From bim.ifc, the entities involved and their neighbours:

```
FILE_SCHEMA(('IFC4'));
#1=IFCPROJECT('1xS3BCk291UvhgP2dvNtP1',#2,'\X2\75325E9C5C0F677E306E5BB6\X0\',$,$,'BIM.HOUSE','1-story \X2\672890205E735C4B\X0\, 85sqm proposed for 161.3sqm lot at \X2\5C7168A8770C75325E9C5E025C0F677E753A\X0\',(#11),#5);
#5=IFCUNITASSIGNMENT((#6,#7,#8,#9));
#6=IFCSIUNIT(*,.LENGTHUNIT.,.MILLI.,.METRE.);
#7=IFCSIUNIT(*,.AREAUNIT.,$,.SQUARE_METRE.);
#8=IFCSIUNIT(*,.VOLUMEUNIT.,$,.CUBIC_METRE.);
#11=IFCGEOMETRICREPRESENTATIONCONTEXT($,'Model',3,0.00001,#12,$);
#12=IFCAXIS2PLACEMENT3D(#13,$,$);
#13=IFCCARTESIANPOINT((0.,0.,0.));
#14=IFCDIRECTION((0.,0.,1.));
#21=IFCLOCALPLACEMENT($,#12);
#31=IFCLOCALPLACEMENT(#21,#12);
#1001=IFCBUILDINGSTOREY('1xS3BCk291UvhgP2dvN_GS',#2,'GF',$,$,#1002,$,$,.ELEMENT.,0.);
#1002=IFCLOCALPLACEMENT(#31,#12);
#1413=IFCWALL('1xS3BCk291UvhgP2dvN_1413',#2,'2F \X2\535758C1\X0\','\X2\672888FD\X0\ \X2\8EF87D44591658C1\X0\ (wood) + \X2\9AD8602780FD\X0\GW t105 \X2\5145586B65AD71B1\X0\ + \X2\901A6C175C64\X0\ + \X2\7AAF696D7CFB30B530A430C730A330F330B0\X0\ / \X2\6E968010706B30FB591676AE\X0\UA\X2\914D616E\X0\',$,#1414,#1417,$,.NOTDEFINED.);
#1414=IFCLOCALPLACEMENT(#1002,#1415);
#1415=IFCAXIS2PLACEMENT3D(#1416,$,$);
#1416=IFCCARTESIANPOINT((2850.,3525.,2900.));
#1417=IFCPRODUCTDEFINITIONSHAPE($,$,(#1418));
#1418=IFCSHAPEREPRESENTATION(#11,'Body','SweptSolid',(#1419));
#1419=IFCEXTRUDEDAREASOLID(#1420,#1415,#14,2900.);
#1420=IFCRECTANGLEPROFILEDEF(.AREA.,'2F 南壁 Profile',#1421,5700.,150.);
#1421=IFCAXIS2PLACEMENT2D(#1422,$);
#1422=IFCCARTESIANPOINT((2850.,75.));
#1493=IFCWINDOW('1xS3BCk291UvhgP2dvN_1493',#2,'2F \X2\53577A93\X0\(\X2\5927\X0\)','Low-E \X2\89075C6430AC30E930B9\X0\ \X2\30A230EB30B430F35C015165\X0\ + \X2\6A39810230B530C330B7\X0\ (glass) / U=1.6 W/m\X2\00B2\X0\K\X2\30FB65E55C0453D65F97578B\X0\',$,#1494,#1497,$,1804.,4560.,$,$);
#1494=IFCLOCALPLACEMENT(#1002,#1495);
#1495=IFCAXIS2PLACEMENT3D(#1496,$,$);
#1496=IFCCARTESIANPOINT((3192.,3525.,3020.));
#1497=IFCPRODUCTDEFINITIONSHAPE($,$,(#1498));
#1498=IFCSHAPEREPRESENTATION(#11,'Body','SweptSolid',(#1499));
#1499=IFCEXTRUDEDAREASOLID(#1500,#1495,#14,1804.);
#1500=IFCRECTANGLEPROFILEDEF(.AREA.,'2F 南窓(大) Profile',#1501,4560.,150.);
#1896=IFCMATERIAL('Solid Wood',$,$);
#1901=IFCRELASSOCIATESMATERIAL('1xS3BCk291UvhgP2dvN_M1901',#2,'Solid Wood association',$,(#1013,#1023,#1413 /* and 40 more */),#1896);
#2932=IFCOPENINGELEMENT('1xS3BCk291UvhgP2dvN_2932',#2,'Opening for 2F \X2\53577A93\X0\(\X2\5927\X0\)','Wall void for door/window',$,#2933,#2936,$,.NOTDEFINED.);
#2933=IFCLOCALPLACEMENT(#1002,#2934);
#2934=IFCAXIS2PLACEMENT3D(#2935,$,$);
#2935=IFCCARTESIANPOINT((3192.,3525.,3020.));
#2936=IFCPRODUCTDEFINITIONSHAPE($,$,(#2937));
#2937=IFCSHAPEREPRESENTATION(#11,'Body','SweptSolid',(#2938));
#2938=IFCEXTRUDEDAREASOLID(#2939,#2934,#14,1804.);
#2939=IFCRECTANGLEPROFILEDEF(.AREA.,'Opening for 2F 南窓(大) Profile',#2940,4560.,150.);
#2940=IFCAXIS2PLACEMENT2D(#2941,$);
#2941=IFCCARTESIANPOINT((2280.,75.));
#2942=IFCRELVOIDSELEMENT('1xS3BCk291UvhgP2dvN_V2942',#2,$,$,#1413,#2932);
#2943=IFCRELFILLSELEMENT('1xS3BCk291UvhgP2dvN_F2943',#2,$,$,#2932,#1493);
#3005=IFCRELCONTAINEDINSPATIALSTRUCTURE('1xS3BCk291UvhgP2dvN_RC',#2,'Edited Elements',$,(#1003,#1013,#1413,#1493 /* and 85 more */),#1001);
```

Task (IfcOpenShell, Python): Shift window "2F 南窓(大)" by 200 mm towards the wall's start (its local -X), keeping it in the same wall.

```python
import ifcopenshell
import ifcopenshell.api.geometry
import ifcopenshell.util.placement
import ifcopenshell.util.unit

model = ifcopenshell.open("bim.ifc")
unit_scale = ifcopenshell.util.unit.calculate_unit_scale(model)

window = model.by_guid("1xS3BCk291UvhgP2dvN_1493")
opening = window.FillsVoids[0].RelatingOpeningElement
wall = opening.VoidsElements[0].RelatingBuildingElement

wall_matrix = ifcopenshell.util.placement.get_local_placement(wall.ObjectPlacement)
shift = wall_matrix[:3, 0] * -0.2 / unit_scale
before = ifcopenshell.util.placement.get_local_placement(window.ObjectPlacement)[:3, 3].copy()

# The window is not placed relative to its opening, so move both.
for product in (opening, window):
    matrix = ifcopenshell.util.placement.get_local_placement(product.ObjectPlacement)
    matrix[:3, 3] += shift
    ifcopenshell.api.geometry.edit_object_placement(model, product=product, matrix=matrix, is_si=False)

after = ifcopenshell.util.placement.get_local_placement(window.ObjectPlacement)[:3, 3]
print("window moved by", (after - before).round(3) + 0.0)

model.write("bim_v2.ifc")
```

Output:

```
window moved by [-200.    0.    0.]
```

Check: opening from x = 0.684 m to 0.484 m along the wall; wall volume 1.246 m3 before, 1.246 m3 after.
